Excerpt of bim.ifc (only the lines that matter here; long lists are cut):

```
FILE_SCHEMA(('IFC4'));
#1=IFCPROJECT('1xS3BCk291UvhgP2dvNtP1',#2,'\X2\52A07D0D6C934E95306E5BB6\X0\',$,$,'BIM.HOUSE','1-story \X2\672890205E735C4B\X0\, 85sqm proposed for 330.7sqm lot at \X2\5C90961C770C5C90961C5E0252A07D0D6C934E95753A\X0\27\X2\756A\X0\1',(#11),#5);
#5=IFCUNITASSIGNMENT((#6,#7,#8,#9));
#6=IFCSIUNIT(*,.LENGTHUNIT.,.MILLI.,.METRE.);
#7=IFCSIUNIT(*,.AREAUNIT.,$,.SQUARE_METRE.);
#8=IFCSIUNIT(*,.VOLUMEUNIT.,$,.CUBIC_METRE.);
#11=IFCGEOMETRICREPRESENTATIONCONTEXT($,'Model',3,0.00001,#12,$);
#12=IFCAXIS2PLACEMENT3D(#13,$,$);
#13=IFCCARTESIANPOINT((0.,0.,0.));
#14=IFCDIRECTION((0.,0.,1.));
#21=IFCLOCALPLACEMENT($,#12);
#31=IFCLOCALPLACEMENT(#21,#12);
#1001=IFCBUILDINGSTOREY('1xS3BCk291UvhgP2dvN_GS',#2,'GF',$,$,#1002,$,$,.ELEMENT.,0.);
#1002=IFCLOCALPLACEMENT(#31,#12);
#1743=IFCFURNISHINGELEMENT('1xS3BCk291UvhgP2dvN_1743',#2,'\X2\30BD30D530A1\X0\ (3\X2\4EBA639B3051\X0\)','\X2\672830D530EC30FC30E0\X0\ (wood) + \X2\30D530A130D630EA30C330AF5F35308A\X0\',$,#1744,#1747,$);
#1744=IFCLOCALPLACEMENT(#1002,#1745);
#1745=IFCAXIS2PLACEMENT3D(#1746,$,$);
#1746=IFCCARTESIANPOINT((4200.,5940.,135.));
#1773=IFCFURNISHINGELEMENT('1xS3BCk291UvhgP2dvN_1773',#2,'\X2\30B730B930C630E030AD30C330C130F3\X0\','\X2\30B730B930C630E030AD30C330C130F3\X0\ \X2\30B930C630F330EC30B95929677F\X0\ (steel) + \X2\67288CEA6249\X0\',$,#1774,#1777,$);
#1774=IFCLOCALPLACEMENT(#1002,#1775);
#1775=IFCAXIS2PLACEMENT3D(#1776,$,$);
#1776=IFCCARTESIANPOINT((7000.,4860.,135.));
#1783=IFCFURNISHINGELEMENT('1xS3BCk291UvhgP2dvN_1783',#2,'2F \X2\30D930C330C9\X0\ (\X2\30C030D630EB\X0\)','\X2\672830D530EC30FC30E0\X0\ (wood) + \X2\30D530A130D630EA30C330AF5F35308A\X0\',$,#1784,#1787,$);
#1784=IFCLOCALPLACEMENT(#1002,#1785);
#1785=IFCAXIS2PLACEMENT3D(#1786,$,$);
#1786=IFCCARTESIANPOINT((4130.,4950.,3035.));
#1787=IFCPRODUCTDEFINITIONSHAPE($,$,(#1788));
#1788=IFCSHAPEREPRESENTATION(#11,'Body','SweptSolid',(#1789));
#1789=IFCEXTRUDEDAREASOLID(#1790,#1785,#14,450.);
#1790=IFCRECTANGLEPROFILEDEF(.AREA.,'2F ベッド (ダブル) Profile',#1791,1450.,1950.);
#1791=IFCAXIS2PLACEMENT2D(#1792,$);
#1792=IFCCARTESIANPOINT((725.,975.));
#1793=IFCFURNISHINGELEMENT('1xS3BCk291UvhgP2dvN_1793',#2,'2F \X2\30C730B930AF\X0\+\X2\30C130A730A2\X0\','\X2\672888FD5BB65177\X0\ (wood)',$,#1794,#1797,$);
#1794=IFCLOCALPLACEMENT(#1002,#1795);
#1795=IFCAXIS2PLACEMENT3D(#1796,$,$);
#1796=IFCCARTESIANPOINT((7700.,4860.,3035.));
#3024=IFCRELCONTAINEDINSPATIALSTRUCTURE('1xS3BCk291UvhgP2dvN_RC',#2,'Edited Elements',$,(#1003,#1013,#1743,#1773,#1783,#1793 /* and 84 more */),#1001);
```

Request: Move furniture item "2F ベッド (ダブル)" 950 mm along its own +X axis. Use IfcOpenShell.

```python
import ifcopenshell
import ifcopenshell.api.geometry
import ifcopenshell.util.placement
import ifcopenshell.util.unit

model = ifcopenshell.open("bim.ifc")
unit_scale = ifcopenshell.util.unit.calculate_unit_scale(model)

item = model.by_guid("1xS3BCk291UvhgP2dvN_1783")
matrix = ifcopenshell.util.placement.get_local_placement(item.ObjectPlacement)
matrix[:3, 3] += matrix[:3, 0] * 0.95 / unit_scale
ifcopenshell.api.geometry.edit_object_placement(model, product=item, matrix=matrix, is_si=False)

print(ifcopenshell.util.placement.get_local_placement(item.ObjectPlacement).round(3) + 0.0)

model.write("bim-out.ifc")
```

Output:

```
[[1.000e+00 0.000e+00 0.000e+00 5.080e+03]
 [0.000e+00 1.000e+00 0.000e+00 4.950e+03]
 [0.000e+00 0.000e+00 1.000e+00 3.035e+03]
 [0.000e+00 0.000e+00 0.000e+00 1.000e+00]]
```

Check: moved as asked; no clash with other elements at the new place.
